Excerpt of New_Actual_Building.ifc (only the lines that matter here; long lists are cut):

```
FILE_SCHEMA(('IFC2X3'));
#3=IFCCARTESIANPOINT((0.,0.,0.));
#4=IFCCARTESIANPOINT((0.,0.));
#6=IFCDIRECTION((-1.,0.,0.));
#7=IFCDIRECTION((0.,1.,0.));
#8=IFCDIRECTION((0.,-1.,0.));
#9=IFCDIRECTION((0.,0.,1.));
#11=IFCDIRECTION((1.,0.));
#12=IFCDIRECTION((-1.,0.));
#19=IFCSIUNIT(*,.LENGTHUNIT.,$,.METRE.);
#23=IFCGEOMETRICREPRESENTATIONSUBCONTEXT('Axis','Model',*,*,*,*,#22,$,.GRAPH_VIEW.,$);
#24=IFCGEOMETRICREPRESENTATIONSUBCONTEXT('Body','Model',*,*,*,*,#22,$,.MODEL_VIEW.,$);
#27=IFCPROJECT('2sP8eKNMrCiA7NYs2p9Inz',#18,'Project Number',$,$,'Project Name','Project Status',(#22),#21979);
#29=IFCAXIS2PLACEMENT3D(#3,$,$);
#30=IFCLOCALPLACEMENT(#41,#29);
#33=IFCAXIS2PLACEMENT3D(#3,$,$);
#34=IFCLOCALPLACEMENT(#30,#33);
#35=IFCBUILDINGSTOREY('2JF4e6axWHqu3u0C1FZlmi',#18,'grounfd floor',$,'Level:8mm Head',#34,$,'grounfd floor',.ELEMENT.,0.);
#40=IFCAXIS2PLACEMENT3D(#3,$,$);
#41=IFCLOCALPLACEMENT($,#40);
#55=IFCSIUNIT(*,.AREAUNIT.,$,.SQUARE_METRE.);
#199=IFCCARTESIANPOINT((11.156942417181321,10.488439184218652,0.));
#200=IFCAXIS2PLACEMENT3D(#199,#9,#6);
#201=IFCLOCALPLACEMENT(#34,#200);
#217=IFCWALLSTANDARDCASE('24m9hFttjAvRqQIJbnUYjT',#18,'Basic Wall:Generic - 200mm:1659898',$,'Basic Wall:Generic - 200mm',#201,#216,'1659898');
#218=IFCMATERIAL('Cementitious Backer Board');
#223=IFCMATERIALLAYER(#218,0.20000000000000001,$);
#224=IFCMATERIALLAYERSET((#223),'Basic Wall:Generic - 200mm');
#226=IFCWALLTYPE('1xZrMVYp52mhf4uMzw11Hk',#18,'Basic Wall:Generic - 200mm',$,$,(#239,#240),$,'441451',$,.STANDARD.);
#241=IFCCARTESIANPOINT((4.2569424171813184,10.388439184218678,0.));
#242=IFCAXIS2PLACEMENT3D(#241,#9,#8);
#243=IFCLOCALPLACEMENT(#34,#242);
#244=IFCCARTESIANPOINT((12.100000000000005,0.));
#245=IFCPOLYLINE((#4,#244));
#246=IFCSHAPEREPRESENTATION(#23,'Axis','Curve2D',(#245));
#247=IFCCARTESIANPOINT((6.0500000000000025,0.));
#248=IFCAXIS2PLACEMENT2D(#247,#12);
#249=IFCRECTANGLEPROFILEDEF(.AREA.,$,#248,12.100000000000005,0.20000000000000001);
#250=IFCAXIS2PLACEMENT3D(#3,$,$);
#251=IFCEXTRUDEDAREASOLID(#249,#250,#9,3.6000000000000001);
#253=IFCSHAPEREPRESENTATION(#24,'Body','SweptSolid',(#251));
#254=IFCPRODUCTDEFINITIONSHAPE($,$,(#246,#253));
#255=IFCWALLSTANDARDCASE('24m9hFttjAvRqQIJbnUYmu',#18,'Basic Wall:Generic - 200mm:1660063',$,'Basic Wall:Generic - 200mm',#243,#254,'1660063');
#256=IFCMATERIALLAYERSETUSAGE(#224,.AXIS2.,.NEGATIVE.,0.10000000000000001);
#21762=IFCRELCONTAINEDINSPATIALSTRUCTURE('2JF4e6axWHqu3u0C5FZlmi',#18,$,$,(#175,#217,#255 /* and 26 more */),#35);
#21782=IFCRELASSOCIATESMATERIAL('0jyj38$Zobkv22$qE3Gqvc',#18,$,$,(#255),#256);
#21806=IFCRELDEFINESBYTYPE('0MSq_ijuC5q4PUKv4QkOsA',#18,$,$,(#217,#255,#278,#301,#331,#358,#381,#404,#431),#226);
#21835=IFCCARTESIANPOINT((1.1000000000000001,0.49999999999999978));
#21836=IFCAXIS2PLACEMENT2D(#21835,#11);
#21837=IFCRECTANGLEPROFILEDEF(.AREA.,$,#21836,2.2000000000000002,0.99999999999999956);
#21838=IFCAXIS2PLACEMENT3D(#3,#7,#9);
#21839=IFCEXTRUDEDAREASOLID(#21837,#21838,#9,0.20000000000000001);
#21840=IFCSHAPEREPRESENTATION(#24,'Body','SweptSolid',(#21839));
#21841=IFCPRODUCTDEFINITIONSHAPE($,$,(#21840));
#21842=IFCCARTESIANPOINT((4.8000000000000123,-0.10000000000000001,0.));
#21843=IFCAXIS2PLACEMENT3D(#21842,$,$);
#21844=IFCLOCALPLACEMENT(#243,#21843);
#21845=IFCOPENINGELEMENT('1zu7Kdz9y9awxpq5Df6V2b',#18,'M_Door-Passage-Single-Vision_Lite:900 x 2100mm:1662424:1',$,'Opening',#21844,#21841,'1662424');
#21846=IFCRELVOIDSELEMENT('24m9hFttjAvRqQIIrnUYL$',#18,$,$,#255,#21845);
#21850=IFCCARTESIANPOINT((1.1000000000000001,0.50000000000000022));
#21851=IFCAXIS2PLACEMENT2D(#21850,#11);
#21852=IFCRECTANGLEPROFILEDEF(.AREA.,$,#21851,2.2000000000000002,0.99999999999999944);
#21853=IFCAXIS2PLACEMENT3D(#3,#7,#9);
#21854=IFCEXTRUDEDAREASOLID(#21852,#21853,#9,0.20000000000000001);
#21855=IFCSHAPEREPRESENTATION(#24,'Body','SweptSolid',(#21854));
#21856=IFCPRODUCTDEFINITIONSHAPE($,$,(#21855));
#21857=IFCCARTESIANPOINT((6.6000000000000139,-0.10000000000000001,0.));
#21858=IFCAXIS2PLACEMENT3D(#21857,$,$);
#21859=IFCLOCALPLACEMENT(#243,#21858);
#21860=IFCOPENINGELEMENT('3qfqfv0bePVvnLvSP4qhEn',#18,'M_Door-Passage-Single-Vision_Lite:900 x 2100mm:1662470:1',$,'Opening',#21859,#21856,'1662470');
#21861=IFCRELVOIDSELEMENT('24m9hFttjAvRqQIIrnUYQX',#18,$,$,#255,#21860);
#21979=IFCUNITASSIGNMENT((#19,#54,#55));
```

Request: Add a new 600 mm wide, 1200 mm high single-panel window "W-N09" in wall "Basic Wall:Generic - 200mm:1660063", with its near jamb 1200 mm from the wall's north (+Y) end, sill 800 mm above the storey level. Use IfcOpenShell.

```python
import numpy as np
import ifcopenshell
import ifcopenshell.api.feature
import ifcopenshell.api.geometry
import ifcopenshell.api.root
import ifcopenshell.api.spatial
import ifcopenshell.api.type
import ifcopenshell.geom
import ifcopenshell.util.element
import ifcopenshell.util.placement
import ifcopenshell.util.representation
import ifcopenshell.util.shape
import ifcopenshell.util.unit

model = ifcopenshell.open("New_Actual_Building.ifc")
unit_scale = ifcopenshell.util.unit.calculate_unit_scale(model)
settings = ifcopenshell.geom.settings()


def volume(element):
    """Net volume in cubic metres, openings subtracted."""
    shape = ifcopenshell.geom.create_shape(settings, element)
    return ifcopenshell.util.shape.get_volume(shape.geometry)


wall = model.by_guid("24m9hFttjAvRqQIJbnUYmu")
storey = ifcopenshell.util.element.get_container(wall, ifc_class="IfcBuildingStorey")
context = ifcopenshell.util.representation.get_context(model, "Model", "Body", "MODEL_VIEW")
before = volume(wall)

width, height, from_end, sill = 0.6, 1.2, 1.2, 0.8  # metres

# The wall runs along its own X axis, and the end named is its -X end.
wall_shape = ifcopenshell.geom.create_shape(settings, wall)
x, y, z = ifcopenshell.util.shape.get_vertices(wall_shape.geometry).T
start = x.min() + from_end
face, thickness = float(y.min()), float(y.max() - y.min())
wall_matrix = ifcopenshell.util.placement.get_local_placement(wall.ObjectPlacement)
level = ifcopenshell.util.placement.get_local_placement(storey.ObjectPlacement)[2, 3]


def in_wall(x, y):
    """Placement at x, y metres in the wall's axes, at sill height."""
    matrix = wall_matrix.copy()
    matrix[:, 3] = wall_matrix @ np.array([x / unit_scale, y / unit_scale, 0.0, 1.0])
    matrix[2, 3] = level + sill / unit_scale
    return matrix


# Opening: a box that overshoots both wall faces by 50 mm.
opening = ifcopenshell.api.root.create_entity(model, ifc_class="IfcOpeningElement")
box = ifcopenshell.api.geometry.add_wall_representation(
    model, context=context, length=width, height=height, thickness=thickness + 0.1
)
ifcopenshell.api.geometry.assign_representation(model, product=opening, representation=box)
ifcopenshell.api.geometry.edit_object_placement(model, product=opening, matrix=in_wall(start, face - 0.05), is_si=False)
ifcopenshell.api.feature.add_feature(model, feature=opening, element=wall)

window = ifcopenshell.api.root.create_entity(model, ifc_class="IfcWindow", name="W-N09")
window.OverallWidth, window.OverallHeight = width / unit_scale, height / unit_scale
body = ifcopenshell.api.geometry.add_window_representation(
    model,
    context=context,
    overall_width=window.OverallWidth,
    overall_height=window.OverallHeight,
    partition_type="SINGLE_PANEL",
)
ifcopenshell.api.geometry.assign_representation(model, product=window, representation=body)
ifcopenshell.api.spatial.assign_container(model, products=[window], relating_structure=storey)
fills = ifcopenshell.api.feature.add_filling(model, opening=opening, element=window)
fills.OwnerHistory = window.OwnerHistory  # required in IFC2X3

# IFC2X3 keeps the operation on the window style.
style = ifcopenshell.api.root.create_entity(model, ifc_class="IfcWindowStyle", name="W-N09")
style.OperationType, style.ConstructionType = "SINGLE_PANEL", "NOTDEFINED"
style.ParameterTakesPrecedence = style.Sizeable = False
ifcopenshell.api.type.assign_type(model, related_objects=[window], relating_type=style)

# Centre the window in the wall's thickness.
ifcopenshell.api.geometry.edit_object_placement(model, product=window, matrix=in_wall(start, face), is_si=False)
window_shape = ifcopenshell.geom.create_shape(settings, window)
depth = ifcopenshell.util.shape.get_vertices(window_shape.geometry)[:, 1]
offset = face + thickness / 2 - (depth.min() + depth.max()) / 2
ifcopenshell.api.geometry.edit_object_placement(model, product=window, matrix=in_wall(start, offset), is_si=False)

after = volume(wall)

print(f"wall volume {before:.3f} -> {after:.3f} m3")

model.write("New_Actual_Building_rev.ifc")
```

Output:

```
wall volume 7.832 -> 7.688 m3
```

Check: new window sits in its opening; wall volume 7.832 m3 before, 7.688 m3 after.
